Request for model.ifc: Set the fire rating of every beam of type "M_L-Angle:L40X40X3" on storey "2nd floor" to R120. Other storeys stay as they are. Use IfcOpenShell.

First a look at what the model holds.

```python
import ifcopenshell
import ifcopenshell.util.element

model = ifcopenshell.open("model.ifc")
print(model.schema)
storey = next(s for s in model.by_type("IfcBuildingStorey") if s.Name == "2nd floor")
beams = [e for e in ifcopenshell.util.element.get_decomposition(storey) if e.is_a("IfcBeam")]
seen = {}
for e in beams:
    element_type = ifcopenshell.util.element.get_type(e)
    key = (element_type.Name if element_type != e and element_type else None, ifcopenshell.util.element.get_pset(e, "Pset_BeamCommon", "FireRating"))
    seen[key] = seen.get(key, 0) + 1
for (name, value), count in sorted(seen.items(), key=str):
    print(count, "x", name, "|", value)
```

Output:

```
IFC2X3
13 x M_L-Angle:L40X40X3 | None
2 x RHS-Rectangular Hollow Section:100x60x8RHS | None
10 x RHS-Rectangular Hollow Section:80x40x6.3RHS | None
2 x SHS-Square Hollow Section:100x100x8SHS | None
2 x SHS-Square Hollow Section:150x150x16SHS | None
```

```python
import ifcopenshell
import ifcopenshell.api.pset
import ifcopenshell.util.element

model = ifcopenshell.open("model.ifc")

storey = next(s for s in model.by_type("IfcBuildingStorey") if s.Name == "2nd floor")
beams = [e for e in ifcopenshell.util.element.get_decomposition(storey) if e.is_a("IfcBeam")]

count = 0
for e in beams:
    element_type = ifcopenshell.util.element.get_type(e)
    if element_type in (None, e) or element_type.Name != "M_L-Angle:L40X40X3":
        continue
    # add_pset returns the element's existing set when there is one.
    pset = ifcopenshell.api.pset.add_pset(model, product=e, name="Pset_BeamCommon")
    ifcopenshell.api.pset.edit_pset(model, pset=pset, properties={"FireRating": "R120"})
    count += 1

print(count, "beams updated")

model.write("model_edited.ifc")
```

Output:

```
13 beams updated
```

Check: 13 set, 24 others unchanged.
